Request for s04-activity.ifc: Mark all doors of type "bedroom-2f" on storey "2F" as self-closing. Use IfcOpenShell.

First a look at what the model holds.

```python
import ifcopenshell
import ifcopenshell.util.element

model = ifcopenshell.open("s04-activity.ifc")
print(model.schema)
storey = next(s for s in model.by_type("IfcBuildingStorey") if s.Name == "2F")
doors = [e for e in ifcopenshell.util.element.get_decomposition(storey) if e.is_a("IfcDoor")]
seen = {}
for e in doors:
    element_type = ifcopenshell.util.element.get_type(e)
    key = (element_type.Name if element_type != e and element_type else None, ifcopenshell.util.element.get_pset(e, "Pset_DoorCommon", "SelfClosing"))
    seen[key] = seen.get(key, 0) + 1
for (name, value), count in sorted(seen.items(), key=str):
    print(count, "x", name, "|", value)
```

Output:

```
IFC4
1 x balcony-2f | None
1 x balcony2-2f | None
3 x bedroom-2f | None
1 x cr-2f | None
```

```python
import ifcopenshell
import ifcopenshell.api.pset
import ifcopenshell.util.element

model = ifcopenshell.open("s04-activity.ifc")

storey = next(s for s in model.by_type("IfcBuildingStorey") if s.Name == "2F")
doors = [e for e in ifcopenshell.util.element.get_decomposition(storey) if e.is_a("IfcDoor")]

count = 0
for e in doors:
    element_type = ifcopenshell.util.element.get_type(e)
    if element_type in (None, e) or element_type.Name != "bedroom-2f":
        continue
    # add_pset returns the element's existing set when there is one.
    pset = ifcopenshell.api.pset.add_pset(model, product=e, name="Pset_DoorCommon")
    ifcopenshell.api.pset.edit_pset(model, pset=pset, properties={"SelfClosing": True})
    count += 1

print(count, "doors updated")

model.write("s04-activity_rev.ifc")
```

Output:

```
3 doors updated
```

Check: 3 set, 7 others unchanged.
